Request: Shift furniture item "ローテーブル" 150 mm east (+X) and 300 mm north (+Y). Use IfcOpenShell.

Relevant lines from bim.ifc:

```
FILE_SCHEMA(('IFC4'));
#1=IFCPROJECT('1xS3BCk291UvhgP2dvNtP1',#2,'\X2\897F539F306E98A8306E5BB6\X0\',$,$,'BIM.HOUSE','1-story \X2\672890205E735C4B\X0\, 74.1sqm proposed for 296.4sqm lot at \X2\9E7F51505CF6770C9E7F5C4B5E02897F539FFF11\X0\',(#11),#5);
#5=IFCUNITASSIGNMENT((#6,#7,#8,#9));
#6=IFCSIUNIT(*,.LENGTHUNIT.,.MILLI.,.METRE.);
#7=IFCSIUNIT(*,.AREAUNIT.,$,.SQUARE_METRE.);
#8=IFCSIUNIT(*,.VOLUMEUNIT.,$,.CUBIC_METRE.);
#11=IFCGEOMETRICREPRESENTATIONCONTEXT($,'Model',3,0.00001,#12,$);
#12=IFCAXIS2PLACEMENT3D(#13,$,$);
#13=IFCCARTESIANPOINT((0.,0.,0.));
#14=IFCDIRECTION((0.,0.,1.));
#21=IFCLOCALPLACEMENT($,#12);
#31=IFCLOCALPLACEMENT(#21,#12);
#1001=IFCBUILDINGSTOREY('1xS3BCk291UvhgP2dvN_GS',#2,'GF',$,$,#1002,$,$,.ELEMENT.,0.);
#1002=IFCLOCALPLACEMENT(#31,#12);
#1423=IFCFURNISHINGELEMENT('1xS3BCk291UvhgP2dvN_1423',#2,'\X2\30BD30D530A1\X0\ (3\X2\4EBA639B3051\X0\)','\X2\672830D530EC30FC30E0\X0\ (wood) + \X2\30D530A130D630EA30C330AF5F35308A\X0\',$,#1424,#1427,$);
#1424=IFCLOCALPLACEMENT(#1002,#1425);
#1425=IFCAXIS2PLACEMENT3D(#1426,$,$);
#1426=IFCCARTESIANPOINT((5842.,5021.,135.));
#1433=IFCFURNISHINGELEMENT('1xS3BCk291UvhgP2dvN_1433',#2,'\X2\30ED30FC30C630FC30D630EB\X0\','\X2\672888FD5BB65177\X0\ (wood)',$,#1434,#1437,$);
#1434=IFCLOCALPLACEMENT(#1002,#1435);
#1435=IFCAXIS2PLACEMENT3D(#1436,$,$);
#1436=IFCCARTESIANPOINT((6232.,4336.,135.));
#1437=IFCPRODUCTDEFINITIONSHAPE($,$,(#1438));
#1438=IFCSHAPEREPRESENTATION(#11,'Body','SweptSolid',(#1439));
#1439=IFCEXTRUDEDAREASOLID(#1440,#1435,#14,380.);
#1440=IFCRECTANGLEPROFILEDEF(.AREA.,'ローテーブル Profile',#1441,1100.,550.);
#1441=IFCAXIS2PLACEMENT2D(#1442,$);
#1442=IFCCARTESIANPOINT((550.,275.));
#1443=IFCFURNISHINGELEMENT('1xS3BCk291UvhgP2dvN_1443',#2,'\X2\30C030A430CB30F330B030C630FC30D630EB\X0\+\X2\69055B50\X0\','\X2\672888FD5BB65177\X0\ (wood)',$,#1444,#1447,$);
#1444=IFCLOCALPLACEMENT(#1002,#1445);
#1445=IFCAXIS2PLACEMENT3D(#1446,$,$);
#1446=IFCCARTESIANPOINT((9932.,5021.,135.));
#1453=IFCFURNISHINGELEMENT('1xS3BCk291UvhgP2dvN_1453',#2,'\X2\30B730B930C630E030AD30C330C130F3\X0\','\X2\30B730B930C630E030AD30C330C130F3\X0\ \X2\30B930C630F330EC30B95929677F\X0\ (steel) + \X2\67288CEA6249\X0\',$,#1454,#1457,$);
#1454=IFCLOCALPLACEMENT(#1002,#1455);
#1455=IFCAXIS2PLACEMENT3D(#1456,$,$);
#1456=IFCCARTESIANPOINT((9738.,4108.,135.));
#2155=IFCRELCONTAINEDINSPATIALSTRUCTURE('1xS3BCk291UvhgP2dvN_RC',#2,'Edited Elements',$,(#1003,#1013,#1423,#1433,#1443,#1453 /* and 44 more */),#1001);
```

```python
import ifcopenshell
import ifcopenshell.api.geometry
import ifcopenshell.util.placement
import ifcopenshell.util.unit

model = ifcopenshell.open("bim.ifc")
unit_scale = ifcopenshell.util.unit.calculate_unit_scale(model)

item = model.by_guid("1xS3BCk291UvhgP2dvN_1433")
matrix = ifcopenshell.util.placement.get_local_placement(item.ObjectPlacement)
matrix[0, 3] += 0.15 / unit_scale
matrix[1, 3] += 0.3 / unit_scale
ifcopenshell.api.geometry.edit_object_placement(model, product=item, matrix=matrix, is_si=False)

print(ifcopenshell.util.placement.get_local_placement(item.ObjectPlacement).round(3) + 0.0)

model.write("bim-out.ifc")
```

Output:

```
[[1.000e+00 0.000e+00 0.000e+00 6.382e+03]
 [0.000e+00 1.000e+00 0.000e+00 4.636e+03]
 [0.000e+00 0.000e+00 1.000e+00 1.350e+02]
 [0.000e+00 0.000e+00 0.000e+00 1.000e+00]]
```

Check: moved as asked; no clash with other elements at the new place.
